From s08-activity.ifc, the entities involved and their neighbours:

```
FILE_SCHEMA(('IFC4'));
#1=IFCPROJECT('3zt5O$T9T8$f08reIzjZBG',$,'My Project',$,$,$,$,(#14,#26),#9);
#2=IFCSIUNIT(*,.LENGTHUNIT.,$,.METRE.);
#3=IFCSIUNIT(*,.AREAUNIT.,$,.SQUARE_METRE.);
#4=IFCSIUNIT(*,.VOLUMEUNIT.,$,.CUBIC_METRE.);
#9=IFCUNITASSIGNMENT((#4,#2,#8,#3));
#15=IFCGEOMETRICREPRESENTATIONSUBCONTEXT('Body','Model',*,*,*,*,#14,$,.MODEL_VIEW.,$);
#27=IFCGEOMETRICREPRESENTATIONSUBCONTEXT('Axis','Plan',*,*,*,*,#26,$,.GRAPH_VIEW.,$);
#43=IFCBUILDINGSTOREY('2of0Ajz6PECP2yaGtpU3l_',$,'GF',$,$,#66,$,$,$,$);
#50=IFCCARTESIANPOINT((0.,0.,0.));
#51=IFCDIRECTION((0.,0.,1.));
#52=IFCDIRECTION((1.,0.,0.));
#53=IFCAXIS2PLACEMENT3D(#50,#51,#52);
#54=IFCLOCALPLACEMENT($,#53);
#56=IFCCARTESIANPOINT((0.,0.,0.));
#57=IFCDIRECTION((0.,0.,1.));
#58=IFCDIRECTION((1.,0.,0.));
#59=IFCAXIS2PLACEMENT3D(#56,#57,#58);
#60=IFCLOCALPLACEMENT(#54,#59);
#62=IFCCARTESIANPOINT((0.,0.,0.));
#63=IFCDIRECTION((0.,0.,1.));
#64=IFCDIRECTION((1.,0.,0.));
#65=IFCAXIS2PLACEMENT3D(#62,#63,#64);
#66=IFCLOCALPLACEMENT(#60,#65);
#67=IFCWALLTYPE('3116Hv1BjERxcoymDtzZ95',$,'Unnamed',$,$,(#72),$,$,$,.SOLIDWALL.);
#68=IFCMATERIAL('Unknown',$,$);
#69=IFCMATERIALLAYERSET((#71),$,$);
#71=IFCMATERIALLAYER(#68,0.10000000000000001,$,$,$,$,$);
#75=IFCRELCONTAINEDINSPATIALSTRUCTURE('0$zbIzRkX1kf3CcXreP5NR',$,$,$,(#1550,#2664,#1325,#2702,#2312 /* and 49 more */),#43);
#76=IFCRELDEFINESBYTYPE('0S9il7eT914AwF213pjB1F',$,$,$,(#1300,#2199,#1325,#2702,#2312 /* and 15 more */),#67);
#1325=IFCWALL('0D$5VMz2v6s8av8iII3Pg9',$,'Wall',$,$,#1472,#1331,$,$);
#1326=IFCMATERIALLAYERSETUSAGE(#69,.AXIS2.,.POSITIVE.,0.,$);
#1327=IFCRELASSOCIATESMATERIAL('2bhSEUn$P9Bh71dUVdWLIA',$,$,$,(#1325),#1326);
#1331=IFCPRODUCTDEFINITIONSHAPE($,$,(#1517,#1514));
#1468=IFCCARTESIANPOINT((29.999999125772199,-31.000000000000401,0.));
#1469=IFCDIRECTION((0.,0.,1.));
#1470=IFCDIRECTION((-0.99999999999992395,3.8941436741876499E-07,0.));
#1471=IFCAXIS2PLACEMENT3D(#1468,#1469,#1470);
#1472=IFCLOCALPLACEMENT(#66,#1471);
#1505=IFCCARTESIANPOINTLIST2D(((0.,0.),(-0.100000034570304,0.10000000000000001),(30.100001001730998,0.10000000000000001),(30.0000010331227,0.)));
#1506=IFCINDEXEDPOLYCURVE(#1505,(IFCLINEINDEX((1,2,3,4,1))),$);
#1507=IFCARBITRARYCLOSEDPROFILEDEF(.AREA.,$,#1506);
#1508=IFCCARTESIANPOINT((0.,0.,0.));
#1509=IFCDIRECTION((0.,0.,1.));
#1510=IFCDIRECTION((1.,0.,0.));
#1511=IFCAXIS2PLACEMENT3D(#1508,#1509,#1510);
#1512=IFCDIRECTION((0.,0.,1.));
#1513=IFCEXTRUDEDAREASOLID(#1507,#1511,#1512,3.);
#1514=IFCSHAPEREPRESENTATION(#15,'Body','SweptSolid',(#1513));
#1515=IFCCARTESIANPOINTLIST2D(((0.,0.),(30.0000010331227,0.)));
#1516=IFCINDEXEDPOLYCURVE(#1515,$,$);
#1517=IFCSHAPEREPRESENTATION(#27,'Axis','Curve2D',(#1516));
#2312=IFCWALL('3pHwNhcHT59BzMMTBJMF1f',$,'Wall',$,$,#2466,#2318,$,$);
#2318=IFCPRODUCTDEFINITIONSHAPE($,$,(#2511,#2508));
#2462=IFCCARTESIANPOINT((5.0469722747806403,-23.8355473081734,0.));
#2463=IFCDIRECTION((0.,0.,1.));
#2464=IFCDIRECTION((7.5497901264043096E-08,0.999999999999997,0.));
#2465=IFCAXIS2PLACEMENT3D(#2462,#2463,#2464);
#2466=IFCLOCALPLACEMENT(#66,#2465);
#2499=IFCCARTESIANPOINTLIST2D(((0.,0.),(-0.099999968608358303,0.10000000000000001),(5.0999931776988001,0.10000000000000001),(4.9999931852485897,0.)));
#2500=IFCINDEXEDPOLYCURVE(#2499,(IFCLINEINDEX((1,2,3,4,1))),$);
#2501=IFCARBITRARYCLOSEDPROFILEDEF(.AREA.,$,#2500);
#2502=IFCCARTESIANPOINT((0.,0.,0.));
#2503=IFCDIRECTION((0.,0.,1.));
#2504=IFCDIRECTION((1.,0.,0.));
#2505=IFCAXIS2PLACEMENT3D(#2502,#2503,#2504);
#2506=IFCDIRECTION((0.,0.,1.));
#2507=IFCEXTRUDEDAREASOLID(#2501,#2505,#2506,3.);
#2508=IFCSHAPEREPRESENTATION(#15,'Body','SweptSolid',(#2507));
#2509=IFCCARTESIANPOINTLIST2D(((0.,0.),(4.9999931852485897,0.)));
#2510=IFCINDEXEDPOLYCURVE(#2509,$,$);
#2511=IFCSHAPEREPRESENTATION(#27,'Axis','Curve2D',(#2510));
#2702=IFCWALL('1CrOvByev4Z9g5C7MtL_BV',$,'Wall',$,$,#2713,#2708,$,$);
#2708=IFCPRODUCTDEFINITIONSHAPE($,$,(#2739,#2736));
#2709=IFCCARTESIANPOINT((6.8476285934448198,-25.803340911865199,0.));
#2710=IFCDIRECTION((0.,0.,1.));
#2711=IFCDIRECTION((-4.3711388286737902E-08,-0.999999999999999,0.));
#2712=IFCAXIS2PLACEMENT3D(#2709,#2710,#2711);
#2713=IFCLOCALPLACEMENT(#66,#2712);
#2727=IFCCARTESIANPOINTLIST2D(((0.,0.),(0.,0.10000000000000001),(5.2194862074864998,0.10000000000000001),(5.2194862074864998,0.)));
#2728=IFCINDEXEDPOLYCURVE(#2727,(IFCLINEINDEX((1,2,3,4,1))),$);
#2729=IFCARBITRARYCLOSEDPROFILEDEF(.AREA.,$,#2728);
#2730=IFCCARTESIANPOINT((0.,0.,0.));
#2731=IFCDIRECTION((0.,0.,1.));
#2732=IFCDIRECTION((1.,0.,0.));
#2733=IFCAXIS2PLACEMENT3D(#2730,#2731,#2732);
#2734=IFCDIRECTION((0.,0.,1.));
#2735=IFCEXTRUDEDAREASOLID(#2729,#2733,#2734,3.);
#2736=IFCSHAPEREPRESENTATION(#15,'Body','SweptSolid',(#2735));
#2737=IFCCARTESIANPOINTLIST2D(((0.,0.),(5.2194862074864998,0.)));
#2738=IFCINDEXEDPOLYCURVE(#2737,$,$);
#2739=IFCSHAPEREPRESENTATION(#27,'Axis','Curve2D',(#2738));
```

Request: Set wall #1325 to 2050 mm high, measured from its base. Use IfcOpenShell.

```python
import ifcopenshell
import ifcopenshell.geom
import ifcopenshell.util.representation
import ifcopenshell.util.shape
import ifcopenshell.util.unit

model = ifcopenshell.open("s08-activity.ifc")
unit_scale = ifcopenshell.util.unit.calculate_unit_scale(model)
settings = ifcopenshell.geom.settings()


def volume(element):
    """Net volume in cubic metres, openings subtracted."""
    shape = ifcopenshell.geom.create_shape(settings, element)
    return ifcopenshell.util.shape.get_volume(shape.geometry)


wall = model.by_id(1325)
before = volume(wall)

body = ifcopenshell.util.representation.get_representation(wall, "Model", "Body")
solid = body.Items[0]
old_height = solid.Depth
solid.Depth = 2.05 / unit_scale
after = volume(wall)

print(f"height {old_height:g} -> {solid.Depth:g}, volume {before:.3f} -> {after:.3f} m3")

model.write("s08-activity_v2.ifc")
```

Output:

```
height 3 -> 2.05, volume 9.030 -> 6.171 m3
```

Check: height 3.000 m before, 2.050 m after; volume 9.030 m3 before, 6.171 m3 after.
